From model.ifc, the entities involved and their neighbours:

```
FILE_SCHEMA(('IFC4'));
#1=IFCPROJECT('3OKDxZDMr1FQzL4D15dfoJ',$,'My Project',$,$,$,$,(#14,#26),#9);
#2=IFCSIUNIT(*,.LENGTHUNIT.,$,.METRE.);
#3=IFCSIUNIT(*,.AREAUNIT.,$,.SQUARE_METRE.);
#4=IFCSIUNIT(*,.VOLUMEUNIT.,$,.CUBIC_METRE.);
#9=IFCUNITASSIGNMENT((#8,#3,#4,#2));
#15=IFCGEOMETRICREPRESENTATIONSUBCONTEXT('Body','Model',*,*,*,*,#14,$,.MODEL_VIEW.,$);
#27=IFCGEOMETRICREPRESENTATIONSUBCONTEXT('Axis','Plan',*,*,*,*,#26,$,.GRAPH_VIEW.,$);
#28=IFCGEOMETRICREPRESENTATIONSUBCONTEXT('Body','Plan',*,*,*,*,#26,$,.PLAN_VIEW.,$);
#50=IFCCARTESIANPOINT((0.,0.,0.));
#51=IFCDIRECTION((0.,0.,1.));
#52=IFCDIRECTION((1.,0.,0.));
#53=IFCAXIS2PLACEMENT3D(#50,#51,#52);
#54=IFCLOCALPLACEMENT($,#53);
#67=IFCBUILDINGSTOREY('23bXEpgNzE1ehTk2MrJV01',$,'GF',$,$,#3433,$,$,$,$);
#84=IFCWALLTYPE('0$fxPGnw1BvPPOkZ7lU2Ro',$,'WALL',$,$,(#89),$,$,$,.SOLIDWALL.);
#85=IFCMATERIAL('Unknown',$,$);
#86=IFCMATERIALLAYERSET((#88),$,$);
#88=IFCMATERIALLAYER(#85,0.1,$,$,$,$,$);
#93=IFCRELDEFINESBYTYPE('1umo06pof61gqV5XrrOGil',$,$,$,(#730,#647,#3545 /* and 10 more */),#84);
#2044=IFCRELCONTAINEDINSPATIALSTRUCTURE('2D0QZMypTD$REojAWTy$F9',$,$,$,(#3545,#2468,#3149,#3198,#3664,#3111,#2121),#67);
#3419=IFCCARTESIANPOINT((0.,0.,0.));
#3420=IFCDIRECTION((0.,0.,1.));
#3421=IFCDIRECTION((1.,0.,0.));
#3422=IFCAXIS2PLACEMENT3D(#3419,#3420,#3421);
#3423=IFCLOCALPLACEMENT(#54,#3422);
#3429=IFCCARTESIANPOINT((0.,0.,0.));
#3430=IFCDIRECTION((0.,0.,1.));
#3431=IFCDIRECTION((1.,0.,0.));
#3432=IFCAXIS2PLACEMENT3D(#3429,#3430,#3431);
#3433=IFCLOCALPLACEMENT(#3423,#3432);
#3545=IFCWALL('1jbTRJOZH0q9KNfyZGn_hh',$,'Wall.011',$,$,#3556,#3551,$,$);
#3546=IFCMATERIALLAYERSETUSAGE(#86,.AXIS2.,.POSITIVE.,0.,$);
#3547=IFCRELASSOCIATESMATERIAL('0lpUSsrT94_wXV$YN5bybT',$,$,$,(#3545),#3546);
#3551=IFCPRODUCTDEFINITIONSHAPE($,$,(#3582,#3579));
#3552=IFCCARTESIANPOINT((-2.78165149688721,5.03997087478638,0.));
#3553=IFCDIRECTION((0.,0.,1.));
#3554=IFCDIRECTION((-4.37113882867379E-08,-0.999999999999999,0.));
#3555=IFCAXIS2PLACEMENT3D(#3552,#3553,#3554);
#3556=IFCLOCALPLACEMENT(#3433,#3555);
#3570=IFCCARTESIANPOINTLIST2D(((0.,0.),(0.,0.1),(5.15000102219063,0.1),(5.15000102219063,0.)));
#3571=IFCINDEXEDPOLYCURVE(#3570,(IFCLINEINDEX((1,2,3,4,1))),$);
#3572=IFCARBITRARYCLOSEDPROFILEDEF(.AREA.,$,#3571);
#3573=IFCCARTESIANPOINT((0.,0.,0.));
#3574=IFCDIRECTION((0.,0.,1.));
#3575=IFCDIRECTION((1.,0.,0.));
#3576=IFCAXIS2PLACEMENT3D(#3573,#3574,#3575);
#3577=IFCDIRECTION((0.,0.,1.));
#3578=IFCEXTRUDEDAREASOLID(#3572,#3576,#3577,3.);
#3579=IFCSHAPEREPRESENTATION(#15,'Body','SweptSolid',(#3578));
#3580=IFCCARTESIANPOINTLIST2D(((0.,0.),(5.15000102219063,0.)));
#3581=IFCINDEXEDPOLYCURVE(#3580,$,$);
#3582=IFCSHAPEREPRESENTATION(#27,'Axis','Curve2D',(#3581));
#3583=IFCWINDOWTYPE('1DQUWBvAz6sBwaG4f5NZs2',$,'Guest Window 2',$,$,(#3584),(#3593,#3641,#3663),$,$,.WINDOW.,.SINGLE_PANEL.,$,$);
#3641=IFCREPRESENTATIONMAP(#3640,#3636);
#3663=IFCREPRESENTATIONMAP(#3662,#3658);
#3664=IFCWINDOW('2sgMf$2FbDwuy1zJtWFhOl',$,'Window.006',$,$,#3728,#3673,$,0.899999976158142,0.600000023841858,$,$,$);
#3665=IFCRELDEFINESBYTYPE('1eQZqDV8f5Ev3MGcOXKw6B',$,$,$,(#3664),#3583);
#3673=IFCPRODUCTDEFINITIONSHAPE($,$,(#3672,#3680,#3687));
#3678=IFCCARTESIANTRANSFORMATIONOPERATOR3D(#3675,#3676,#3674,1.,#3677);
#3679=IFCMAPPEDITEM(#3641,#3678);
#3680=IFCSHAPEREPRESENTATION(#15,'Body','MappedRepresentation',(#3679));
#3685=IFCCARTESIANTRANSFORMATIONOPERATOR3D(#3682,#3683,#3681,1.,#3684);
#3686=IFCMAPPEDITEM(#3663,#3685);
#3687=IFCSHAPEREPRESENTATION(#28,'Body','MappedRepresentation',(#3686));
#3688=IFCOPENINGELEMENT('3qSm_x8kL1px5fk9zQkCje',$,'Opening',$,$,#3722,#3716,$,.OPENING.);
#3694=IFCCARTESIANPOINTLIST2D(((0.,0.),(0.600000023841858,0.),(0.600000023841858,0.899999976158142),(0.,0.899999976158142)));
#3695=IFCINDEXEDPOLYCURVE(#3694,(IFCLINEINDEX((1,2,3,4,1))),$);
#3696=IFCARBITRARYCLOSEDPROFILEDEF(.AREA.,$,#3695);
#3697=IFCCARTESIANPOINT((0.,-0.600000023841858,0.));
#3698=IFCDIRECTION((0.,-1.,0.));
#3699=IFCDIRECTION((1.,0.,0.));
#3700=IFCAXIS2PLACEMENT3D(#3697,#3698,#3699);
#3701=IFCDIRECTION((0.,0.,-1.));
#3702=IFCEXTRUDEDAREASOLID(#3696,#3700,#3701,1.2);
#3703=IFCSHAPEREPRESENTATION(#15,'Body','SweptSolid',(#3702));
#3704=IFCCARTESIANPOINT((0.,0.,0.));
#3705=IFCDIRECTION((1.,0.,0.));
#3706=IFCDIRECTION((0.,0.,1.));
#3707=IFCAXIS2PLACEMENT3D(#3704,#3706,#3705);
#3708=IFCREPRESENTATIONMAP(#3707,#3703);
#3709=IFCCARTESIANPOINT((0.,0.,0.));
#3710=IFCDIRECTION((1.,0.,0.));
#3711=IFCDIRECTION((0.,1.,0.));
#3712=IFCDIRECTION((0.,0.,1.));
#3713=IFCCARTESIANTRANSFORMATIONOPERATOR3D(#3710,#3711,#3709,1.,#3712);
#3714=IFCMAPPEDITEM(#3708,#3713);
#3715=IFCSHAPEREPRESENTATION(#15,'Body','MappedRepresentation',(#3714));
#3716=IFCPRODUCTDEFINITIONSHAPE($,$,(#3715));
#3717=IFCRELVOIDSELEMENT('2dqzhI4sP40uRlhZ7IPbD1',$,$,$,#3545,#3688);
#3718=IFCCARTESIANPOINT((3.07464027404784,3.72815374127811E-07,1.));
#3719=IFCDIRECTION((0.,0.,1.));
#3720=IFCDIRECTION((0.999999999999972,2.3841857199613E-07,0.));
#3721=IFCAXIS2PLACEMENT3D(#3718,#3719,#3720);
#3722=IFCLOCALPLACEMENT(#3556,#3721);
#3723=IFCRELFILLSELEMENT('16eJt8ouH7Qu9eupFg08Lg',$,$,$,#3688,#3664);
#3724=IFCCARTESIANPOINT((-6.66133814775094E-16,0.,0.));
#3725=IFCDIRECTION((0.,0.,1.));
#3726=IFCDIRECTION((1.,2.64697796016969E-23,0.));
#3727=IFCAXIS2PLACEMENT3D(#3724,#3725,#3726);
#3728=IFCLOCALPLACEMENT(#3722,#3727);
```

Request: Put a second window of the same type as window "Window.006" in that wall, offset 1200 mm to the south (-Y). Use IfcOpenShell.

```python
import ifcopenshell
import ifcopenshell.api.feature
import ifcopenshell.api.geometry
import ifcopenshell.api.root
import ifcopenshell.geom
import ifcopenshell.util.element
import ifcopenshell.util.placement
import ifcopenshell.util.shape

model = ifcopenshell.open("model.ifc")
settings = ifcopenshell.geom.settings()


def volume(element):
    """Net volume in cubic metres, openings subtracted."""
    shape = ifcopenshell.geom.create_shape(settings, element)
    return ifcopenshell.util.shape.get_volume(shape.geometry)


window = model.by_guid("2sgMf$2FbDwuy1zJtWFhOl")
opening = window.FillsVoids[0].RelatingOpeningElement
wall = opening.VoidsElements[0].RelatingBuildingElement
before = volume(wall)
shift = ifcopenshell.util.placement.get_local_placement(wall.ObjectPlacement)[:3, 0] * 1.2

# copy_class copies the void relationship, type, container and properties, but no geometry.
new_opening = ifcopenshell.api.root.copy_class(model, product=opening)
new_opening.Representation = ifcopenshell.util.element.copy_deep(
    model, opening.Representation, exclude=["IfcGeometricRepresentationContext", "IfcRepresentationMap"]
)
new_window = ifcopenshell.api.root.copy_class(model, product=window)
new_window.Representation = ifcopenshell.util.element.copy_deep(
    model, window.Representation, exclude=["IfcGeometricRepresentationContext", "IfcRepresentationMap"]
)
ifcopenshell.api.feature.add_filling(model, opening=new_opening, element=new_window)

for old, new in ((opening, new_opening), (window, new_window)):
    matrix = ifcopenshell.util.placement.get_local_placement(old.ObjectPlacement)
    matrix[:3, 3] += shift
    ifcopenshell.api.geometry.edit_object_placement(model, product=new, matrix=matrix, is_si=False)

after = volume(wall)

print(f"wall volume {before:.3f} -> {after:.3f} m3")

model.write("model_edited.ifc")
```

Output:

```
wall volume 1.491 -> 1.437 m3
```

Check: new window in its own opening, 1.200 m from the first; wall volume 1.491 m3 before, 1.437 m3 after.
